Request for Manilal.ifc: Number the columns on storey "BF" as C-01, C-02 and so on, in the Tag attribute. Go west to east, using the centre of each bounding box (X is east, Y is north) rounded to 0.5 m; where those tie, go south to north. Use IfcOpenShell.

First a look at what the model holds.

```python
import ifcopenshell
import ifcopenshell.util.element
import ifcopenshell.util.placement

model = ifcopenshell.open("Manilal.ifc")
print(model.schema)
storey = next(s for s in model.by_type("IfcBuildingStorey") if s.Name == "BF")
columns = [e for e in ifcopenshell.util.element.get_decomposition(storey) if e.is_a("IfcColumn")]
for e in sorted(columns, key=lambda e: e.id()):
    origin = ifcopenshell.util.placement.get_local_placement(e.ObjectPlacement)[:3, 3]
    print(e.id(), e.Tag, e.Name, origin.round(2) + 0.0, sep=" | ")
```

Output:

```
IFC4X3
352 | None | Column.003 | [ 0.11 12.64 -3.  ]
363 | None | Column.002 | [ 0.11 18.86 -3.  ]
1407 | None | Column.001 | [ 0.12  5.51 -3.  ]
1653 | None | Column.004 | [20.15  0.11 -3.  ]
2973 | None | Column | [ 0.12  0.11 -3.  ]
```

```python
import ifcopenshell
import ifcopenshell.geom
import ifcopenshell.util.element
import ifcopenshell.util.shape

model = ifcopenshell.open("Manilal.ifc")
settings = ifcopenshell.geom.settings()
settings.set("use-world-coords", True)


def centre(element):
    shape = ifcopenshell.geom.create_shape(settings, element)
    return ifcopenshell.util.shape.get_bbox_centroid(shape.geometry)


storey = next(s for s in model.by_type("IfcBuildingStorey") if s.Name == "BF")
columns = [e for e in ifcopenshell.util.element.get_decomposition(storey) if e.is_a("IfcColumn")]

# Insertion points can sit at a corner or the storey origin, so sort by the geometry (in metres).
centres = {e: centre(e) for e in columns}
columns.sort(key=lambda e: (round(centres[e][0] / 0.5), centres[e][1]))

for i, e in enumerate(columns, start=1):
    number = f"C-{i:02d}"
    e.Tag = number
    print(e.id(), number)

model.write("Manilal_updated.ifc")
```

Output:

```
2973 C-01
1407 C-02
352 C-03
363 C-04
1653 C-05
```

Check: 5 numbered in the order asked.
